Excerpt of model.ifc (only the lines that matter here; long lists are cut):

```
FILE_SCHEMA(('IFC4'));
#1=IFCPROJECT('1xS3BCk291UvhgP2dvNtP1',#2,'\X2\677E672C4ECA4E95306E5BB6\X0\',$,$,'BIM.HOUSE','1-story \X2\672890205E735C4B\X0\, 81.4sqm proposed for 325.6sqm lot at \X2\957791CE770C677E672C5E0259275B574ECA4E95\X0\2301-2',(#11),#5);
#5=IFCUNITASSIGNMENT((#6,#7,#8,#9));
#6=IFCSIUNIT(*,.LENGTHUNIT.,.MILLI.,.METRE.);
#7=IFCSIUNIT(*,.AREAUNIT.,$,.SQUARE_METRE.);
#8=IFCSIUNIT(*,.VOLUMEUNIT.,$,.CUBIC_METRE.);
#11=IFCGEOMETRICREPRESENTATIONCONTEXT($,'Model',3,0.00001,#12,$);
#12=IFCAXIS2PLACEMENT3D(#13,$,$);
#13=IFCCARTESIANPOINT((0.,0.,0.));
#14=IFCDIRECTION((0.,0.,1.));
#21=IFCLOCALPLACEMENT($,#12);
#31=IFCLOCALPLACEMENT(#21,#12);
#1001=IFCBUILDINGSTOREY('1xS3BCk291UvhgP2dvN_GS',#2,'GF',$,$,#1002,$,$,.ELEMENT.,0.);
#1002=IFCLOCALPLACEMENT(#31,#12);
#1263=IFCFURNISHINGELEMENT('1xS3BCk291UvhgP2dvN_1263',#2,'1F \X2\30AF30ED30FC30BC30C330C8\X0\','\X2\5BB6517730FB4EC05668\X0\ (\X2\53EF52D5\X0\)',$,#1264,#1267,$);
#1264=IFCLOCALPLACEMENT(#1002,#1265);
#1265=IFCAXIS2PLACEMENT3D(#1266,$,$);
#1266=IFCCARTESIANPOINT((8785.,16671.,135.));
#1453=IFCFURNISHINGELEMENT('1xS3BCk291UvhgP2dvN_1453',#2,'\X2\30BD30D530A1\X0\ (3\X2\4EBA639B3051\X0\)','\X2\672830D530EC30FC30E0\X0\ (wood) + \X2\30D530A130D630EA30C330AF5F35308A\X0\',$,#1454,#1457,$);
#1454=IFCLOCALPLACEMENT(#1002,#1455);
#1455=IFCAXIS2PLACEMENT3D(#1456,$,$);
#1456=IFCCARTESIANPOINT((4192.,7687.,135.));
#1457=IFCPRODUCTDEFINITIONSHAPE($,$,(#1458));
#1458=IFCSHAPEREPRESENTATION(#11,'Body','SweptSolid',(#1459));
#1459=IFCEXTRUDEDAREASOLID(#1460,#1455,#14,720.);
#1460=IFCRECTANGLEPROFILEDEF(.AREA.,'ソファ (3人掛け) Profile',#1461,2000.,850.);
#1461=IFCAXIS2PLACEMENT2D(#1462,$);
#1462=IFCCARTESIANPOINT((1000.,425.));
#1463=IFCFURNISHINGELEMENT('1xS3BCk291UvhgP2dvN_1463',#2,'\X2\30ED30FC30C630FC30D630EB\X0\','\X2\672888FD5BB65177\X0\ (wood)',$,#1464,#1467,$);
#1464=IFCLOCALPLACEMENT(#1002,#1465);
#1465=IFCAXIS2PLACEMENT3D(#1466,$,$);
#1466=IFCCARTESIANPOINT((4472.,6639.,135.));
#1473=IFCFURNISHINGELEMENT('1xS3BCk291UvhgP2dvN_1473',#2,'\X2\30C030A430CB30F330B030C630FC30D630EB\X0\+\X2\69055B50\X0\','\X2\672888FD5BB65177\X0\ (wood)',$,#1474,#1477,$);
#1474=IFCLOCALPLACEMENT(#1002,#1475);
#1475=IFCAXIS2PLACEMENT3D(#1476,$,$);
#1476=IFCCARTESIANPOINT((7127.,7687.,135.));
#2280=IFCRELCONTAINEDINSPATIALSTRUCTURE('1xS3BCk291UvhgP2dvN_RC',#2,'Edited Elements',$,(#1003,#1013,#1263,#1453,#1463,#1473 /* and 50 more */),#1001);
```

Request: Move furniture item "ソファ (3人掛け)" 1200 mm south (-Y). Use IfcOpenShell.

```python
import ifcopenshell
import ifcopenshell.api.geometry
import ifcopenshell.util.placement
import ifcopenshell.util.unit

model = ifcopenshell.open("model.ifc")
unit_scale = ifcopenshell.util.unit.calculate_unit_scale(model)

item = model.by_guid("1xS3BCk291UvhgP2dvN_1453")
matrix = ifcopenshell.util.placement.get_local_placement(item.ObjectPlacement)
matrix[1, 3] -= 1.2 / unit_scale
ifcopenshell.api.geometry.edit_object_placement(model, product=item, matrix=matrix, is_si=False)

print(ifcopenshell.util.placement.get_local_placement(item.ObjectPlacement).round(3) + 0.0)

model.write("model_rev.ifc")
```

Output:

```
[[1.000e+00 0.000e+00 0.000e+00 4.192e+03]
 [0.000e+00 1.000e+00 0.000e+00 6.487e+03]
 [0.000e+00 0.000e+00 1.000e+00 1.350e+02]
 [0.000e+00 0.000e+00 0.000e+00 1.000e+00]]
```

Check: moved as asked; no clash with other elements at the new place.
